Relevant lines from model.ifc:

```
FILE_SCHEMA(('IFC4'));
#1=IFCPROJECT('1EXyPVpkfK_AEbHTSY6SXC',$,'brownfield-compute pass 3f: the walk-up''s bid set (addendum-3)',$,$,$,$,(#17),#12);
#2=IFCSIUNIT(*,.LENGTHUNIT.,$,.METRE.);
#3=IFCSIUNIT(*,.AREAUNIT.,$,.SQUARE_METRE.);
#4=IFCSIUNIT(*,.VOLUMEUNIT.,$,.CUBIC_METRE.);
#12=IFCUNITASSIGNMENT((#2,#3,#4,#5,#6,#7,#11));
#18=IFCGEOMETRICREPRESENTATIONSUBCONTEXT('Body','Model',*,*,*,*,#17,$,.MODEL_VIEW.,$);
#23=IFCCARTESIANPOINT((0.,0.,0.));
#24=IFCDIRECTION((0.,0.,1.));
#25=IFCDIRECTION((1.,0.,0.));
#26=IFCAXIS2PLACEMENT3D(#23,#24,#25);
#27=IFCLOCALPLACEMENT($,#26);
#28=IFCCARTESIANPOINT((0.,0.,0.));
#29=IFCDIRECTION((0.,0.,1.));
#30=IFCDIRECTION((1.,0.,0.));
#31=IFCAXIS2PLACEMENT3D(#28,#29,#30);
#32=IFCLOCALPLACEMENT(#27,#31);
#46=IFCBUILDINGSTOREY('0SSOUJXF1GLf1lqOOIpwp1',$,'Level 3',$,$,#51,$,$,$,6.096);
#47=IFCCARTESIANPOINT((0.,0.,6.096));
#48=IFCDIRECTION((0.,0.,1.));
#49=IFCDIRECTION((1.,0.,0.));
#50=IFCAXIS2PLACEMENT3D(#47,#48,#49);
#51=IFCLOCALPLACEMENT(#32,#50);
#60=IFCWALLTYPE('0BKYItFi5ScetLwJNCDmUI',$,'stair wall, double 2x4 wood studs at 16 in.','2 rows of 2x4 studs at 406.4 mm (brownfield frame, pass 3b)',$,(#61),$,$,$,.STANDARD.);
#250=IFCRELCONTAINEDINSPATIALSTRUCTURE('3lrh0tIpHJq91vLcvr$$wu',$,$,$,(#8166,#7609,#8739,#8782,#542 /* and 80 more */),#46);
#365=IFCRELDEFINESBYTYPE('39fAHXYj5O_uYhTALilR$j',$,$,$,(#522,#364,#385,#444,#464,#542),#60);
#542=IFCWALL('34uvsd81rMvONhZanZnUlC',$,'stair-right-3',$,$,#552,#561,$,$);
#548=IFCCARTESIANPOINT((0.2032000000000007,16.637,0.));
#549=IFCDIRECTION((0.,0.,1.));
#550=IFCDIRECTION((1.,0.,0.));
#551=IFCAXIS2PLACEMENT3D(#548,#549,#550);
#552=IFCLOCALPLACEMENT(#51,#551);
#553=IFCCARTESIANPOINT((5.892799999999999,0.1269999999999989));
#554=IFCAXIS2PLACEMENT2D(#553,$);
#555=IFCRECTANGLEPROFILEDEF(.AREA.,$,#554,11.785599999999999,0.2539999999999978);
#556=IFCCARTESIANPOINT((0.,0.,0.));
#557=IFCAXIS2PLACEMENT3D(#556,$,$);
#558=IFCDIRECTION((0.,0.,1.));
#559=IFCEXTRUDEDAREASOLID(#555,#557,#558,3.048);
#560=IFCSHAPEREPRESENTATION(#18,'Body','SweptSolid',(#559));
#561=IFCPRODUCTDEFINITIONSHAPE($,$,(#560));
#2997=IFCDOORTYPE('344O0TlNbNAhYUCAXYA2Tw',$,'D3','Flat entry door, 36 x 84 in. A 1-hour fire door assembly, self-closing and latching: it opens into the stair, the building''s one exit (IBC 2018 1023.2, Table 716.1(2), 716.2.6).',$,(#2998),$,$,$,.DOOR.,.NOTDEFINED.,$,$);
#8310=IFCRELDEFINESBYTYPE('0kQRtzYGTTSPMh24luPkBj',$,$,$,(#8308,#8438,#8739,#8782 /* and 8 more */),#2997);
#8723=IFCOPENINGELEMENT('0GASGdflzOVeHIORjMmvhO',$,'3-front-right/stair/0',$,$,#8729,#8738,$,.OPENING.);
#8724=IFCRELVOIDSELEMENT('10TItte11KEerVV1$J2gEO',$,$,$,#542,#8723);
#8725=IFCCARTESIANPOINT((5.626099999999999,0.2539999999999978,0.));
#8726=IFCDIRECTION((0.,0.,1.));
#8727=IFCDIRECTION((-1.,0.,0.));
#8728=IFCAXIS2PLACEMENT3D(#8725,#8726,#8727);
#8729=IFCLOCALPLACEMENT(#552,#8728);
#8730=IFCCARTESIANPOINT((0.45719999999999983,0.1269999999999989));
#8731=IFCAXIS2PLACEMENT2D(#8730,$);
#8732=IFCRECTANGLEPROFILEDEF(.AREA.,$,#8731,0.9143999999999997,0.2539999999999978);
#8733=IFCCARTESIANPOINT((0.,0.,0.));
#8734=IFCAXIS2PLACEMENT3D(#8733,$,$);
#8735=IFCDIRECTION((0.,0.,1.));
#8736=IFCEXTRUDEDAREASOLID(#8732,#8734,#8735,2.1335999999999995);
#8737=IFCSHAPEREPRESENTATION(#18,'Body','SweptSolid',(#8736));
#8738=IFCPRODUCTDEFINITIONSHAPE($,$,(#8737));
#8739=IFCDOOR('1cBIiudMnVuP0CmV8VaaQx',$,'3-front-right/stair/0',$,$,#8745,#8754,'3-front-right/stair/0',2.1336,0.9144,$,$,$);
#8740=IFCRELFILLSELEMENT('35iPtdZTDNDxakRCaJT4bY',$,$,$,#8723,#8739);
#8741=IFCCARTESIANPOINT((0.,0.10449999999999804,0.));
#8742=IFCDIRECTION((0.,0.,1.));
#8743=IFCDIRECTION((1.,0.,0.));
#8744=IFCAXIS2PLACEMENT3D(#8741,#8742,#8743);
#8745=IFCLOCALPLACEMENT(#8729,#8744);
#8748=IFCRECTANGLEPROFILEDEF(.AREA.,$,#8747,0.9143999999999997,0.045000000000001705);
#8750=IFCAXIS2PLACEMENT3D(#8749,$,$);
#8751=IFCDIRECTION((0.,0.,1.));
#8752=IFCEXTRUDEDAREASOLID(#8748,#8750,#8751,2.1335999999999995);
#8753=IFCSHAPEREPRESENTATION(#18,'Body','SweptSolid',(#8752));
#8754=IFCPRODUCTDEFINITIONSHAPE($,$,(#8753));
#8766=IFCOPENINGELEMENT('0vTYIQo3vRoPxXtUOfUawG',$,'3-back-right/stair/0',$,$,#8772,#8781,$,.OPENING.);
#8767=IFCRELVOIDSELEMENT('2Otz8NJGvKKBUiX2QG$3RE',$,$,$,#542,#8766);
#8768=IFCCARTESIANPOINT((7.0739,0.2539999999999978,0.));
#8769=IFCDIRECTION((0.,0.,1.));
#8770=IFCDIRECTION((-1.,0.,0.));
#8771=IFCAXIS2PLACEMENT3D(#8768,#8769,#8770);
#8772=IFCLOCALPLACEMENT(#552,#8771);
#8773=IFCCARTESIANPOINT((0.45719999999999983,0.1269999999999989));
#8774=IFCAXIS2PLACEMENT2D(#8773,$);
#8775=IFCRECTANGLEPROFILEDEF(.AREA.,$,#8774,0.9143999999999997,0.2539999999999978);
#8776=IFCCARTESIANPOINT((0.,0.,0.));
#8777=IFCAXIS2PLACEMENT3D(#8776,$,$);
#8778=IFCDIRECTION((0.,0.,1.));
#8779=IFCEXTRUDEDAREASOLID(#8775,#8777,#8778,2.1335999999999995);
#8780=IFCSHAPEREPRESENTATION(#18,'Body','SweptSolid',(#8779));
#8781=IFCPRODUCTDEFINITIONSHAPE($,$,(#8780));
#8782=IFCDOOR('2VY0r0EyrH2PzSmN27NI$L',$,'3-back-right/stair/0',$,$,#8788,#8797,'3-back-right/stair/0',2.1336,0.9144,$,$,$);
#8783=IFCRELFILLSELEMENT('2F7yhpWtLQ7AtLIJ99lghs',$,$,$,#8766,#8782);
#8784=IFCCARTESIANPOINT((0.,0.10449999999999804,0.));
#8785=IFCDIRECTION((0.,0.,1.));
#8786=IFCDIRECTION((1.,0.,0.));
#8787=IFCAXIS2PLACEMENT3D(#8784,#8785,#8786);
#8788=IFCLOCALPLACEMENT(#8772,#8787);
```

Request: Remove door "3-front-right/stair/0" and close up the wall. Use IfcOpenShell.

```python
import ifcopenshell
import ifcopenshell.api.feature
import ifcopenshell.api.root
import ifcopenshell.geom
import ifcopenshell.util.shape

model = ifcopenshell.open("model.ifc")
settings = ifcopenshell.geom.settings()


def volume(element):
    """Net volume in cubic metres, openings subtracted."""
    shape = ifcopenshell.geom.create_shape(settings, element)
    return ifcopenshell.util.shape.get_volume(shape.geometry)


door = model.by_guid("1cBIiudMnVuP0CmV8VaaQx")
opening = door.FillsVoids[0].RelatingOpeningElement
wall = opening.VoidsElements[0].RelatingBuildingElement
before = volume(wall)

ifcopenshell.api.root.remove_product(model, product=door)
ifcopenshell.api.feature.remove_feature(model, feature=opening)

after = volume(wall)

print(f"wall volume {before:.3f} -> {after:.3f} m3")

model.write("model-out.ifc")
```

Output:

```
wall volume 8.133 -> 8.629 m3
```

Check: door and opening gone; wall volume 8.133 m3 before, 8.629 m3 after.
